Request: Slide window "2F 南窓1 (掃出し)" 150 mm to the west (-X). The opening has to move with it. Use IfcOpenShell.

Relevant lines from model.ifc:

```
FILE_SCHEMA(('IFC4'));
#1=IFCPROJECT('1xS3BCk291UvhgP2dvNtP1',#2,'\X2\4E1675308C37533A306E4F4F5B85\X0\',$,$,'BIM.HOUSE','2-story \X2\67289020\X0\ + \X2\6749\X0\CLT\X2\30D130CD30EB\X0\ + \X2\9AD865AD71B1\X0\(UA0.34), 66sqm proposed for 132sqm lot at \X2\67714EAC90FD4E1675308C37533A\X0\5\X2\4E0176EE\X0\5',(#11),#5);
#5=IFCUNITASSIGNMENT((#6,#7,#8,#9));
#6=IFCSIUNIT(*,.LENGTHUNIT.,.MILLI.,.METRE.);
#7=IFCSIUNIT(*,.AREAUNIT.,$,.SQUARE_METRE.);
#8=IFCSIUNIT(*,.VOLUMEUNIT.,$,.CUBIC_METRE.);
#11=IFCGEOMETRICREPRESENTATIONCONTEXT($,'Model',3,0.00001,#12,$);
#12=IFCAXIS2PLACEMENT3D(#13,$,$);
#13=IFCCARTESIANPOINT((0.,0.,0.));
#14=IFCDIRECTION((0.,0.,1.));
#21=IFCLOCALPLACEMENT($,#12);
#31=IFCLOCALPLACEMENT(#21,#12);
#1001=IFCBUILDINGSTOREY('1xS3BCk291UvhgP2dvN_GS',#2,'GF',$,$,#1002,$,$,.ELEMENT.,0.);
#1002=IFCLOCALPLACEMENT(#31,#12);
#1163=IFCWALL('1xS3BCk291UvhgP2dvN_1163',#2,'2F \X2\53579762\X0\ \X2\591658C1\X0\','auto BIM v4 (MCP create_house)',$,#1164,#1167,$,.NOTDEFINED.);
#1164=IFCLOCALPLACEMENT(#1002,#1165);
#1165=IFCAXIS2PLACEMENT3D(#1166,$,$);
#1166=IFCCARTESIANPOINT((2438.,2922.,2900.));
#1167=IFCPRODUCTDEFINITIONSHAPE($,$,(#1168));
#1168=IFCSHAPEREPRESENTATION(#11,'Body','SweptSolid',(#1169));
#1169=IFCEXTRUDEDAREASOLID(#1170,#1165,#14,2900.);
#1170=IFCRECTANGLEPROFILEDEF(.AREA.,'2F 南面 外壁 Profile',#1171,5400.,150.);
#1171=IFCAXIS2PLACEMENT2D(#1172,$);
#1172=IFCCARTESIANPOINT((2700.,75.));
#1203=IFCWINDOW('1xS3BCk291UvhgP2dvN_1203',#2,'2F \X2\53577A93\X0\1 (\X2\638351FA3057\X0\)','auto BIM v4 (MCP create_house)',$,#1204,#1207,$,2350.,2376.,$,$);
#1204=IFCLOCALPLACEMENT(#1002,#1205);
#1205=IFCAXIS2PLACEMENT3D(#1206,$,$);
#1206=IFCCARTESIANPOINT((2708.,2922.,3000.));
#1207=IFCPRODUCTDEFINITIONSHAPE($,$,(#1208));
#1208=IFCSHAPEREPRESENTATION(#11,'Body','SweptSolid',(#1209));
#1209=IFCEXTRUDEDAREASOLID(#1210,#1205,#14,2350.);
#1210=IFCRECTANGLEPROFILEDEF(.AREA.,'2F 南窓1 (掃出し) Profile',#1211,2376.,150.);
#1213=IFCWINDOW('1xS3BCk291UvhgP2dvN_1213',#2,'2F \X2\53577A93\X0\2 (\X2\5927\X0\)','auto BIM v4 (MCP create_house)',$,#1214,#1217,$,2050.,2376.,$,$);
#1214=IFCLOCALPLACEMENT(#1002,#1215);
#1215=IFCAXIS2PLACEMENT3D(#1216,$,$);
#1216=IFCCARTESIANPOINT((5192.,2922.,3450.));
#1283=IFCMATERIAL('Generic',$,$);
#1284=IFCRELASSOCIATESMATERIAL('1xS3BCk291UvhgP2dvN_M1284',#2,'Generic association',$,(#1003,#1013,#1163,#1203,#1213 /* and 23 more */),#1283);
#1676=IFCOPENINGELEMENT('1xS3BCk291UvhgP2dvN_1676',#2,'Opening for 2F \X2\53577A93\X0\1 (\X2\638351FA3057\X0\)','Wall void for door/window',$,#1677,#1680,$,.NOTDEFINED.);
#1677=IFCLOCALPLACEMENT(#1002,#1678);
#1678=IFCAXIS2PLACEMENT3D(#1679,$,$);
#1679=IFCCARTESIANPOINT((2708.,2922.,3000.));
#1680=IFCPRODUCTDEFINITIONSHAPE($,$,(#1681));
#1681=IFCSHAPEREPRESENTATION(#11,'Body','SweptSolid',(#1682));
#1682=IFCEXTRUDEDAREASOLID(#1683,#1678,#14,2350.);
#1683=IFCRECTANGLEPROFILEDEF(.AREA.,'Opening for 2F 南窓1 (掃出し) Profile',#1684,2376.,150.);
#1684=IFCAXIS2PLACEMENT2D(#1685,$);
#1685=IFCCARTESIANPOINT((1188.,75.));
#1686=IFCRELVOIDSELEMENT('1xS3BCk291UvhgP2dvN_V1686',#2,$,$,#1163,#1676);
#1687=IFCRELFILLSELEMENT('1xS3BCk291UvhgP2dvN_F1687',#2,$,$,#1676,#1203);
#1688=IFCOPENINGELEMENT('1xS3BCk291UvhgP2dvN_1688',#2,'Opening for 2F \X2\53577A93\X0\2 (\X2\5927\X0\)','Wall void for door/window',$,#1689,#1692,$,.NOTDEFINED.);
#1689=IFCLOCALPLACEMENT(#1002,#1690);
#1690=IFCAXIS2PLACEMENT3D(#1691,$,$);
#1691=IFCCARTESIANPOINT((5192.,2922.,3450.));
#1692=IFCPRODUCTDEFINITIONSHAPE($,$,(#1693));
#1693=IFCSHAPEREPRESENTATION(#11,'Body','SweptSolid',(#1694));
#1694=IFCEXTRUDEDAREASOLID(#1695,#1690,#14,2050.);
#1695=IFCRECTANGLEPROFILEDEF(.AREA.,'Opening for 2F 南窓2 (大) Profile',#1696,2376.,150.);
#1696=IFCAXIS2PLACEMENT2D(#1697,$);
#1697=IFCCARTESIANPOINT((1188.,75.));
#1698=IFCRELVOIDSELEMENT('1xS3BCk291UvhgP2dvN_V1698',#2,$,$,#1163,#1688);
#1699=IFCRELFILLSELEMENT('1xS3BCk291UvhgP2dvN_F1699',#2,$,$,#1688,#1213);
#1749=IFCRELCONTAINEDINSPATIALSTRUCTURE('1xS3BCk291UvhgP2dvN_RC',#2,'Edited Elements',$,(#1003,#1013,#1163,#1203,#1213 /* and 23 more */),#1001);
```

```python
import ifcopenshell
import ifcopenshell.api.geometry
import ifcopenshell.util.placement
import ifcopenshell.util.unit

model = ifcopenshell.open("model.ifc")
unit_scale = ifcopenshell.util.unit.calculate_unit_scale(model)

window = model.by_guid("1xS3BCk291UvhgP2dvN_1203")
opening = window.FillsVoids[0].RelatingOpeningElement
wall = opening.VoidsElements[0].RelatingBuildingElement

wall_matrix = ifcopenshell.util.placement.get_local_placement(wall.ObjectPlacement)
shift = wall_matrix[:3, 0] * -0.15 / unit_scale
before = ifcopenshell.util.placement.get_local_placement(window.ObjectPlacement)[:3, 3].copy()

# The window is not placed relative to its opening, so move both.
for product in (opening, window):
    matrix = ifcopenshell.util.placement.get_local_placement(product.ObjectPlacement)
    matrix[:3, 3] += shift
    ifcopenshell.api.geometry.edit_object_placement(model, product=product, matrix=matrix, is_si=False)

after = ifcopenshell.util.placement.get_local_placement(window.ObjectPlacement)[:3, 3]
print("window moved by", (after - before).round(3) + 0.0)

model.write("model_rev.ifc")
```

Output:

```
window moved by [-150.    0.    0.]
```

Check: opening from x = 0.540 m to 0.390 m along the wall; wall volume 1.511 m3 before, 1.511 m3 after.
